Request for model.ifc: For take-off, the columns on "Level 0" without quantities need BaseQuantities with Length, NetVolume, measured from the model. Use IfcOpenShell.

First a look at what the model holds.

```python
import ifcopenshell
import ifcopenshell.util.element
import ifcopenshell.util.unit

model = ifcopenshell.open("model.ifc")
print(model.schema)
for unit_type in ("LENGTHUNIT", "AREAUNIT", "VOLUMEUNIT"):
    print(unit_type, ifcopenshell.util.unit.calculate_unit_scale(model, unit_type))
storey = next(s for s in model.by_type("IfcBuildingStorey") if s.Name == "Level 0")
columns = [e for e in ifcopenshell.util.element.get_decomposition(storey) if e.is_a("IfcColumn")]
for e in sorted(columns, key=lambda e: e.id()):
    print(e.id(), e.is_a(), e.Name, list(ifcopenshell.util.element.get_psets(e, qtos_only=True)), sep=" | ")
```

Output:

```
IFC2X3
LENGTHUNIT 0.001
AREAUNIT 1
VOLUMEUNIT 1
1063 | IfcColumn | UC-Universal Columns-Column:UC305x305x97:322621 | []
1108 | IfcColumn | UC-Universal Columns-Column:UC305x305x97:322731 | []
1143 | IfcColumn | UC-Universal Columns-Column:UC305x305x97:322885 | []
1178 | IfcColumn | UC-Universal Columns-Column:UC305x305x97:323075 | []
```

```python
import ifcopenshell
import ifcopenshell.api.pset
import ifcopenshell.geom
import ifcopenshell.util.element
import ifcopenshell.util.shape
import ifcopenshell.util.unit

model = ifcopenshell.open("model.ifc")
unit_scale = ifcopenshell.util.unit.calculate_unit_scale(model)
volume_scale = ifcopenshell.util.unit.calculate_unit_scale(model, "VOLUMEUNIT")
settings = ifcopenshell.geom.settings()

storey = next(s for s in model.by_type("IfcBuildingStorey") if s.Name == "Level 0")
columns = [e for e in ifcopenshell.util.element.get_decomposition(storey) if e.is_a("IfcColumn")]

for e in sorted(columns, key=lambda e: e.id()):
    if ifcopenshell.util.element.get_psets(e, qtos_only=True, should_inherit=False):
        continue
    # Geometry comes back in metres, in the element's own axes.
    shape = ifcopenshell.geom.create_shape(settings, e)
    values = {
        "Length": ifcopenshell.util.shape.get_z(shape.geometry) / unit_scale,
        "NetVolume": ifcopenshell.util.shape.get_volume(shape.geometry) / volume_scale,
    }
    qto = ifcopenshell.api.pset.add_qto(model, product=e, name="BaseQuantities")
    ifcopenshell.api.pset.edit_qto(model, qto=qto, properties=values)
    print(e.id(), {k: round(v, 3) for k, v in values.items()})

model.write("model_updated.ifc")
```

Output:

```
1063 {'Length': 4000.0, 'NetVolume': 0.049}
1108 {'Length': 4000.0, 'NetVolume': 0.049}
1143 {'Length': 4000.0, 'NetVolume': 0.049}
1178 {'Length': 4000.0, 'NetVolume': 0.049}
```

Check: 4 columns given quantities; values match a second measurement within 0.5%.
